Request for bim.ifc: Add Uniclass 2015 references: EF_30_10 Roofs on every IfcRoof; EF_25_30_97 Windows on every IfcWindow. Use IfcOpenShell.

First a look at what the model holds.

```python
import ifcopenshell

model = ifcopenshell.open("bim.ifc")
print(model.schema)
print("classifications:", [c.Name for c in model.by_type("IfcClassification")])
for ifc_class in ("IfcDoor", "IfcRoof", "IfcStair", "IfcWall", "IfcWindow"):
    print(ifc_class, len(model.by_type(ifc_class)))
```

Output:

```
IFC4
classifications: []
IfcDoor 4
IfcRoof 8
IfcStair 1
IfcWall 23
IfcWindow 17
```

```python
import ifcopenshell
import ifcopenshell.api.classification

model = ifcopenshell.open("bim.ifc")

system = ifcopenshell.api.classification.add_classification(model, classification="Uniclass 2015")

codes = {
    "IfcRoof": ("EF_30_10", "Roofs"),
    "IfcWindow": ("EF_25_30_97", "Windows"),
}
for ifc_class, (code, name) in codes.items():
    products = model.by_type(ifc_class)
    ifcopenshell.api.classification.add_reference(
        model, products=products, classification=system, identification=code, name=name
    )
    print(code, len(products))

model.write("bim-out.ifc")
```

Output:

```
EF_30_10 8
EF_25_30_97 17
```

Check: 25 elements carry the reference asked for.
